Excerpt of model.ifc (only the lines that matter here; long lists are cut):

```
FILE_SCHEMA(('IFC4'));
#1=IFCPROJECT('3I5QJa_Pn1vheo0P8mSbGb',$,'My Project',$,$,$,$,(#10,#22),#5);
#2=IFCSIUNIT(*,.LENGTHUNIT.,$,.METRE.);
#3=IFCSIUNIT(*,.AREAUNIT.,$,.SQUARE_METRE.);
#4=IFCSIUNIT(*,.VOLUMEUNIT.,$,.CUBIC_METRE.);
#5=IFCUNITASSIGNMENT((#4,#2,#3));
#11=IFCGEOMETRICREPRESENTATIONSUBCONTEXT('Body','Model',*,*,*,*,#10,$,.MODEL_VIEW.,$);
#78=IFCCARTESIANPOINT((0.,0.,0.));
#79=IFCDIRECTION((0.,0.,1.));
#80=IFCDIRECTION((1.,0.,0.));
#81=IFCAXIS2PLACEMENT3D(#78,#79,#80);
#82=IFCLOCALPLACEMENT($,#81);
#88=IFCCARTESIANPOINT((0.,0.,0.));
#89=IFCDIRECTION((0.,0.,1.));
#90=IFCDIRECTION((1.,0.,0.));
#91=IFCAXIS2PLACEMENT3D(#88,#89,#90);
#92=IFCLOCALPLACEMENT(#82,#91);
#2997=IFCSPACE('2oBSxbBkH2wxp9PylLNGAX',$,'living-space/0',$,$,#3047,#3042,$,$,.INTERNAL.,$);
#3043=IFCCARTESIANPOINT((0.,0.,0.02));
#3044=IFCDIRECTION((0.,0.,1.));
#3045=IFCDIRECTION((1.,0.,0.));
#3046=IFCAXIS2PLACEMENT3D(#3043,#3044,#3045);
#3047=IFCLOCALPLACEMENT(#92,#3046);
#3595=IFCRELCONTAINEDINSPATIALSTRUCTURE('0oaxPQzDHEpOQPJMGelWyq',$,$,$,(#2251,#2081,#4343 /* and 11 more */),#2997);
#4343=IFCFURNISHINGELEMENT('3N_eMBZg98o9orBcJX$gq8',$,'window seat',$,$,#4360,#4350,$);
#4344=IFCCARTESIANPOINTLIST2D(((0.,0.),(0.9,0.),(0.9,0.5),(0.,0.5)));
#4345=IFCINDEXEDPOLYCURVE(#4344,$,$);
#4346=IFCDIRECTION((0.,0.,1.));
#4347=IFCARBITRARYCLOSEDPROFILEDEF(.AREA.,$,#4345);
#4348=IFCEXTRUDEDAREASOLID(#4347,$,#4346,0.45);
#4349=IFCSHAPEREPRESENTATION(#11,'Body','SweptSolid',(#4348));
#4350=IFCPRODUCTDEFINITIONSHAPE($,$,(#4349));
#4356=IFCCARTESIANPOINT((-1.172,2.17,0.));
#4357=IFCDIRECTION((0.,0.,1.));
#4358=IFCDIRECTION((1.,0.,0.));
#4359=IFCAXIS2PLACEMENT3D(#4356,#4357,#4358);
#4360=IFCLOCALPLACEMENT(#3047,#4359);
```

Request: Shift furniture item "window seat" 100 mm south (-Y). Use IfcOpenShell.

```python
import ifcopenshell
import ifcopenshell.api.geometry
import ifcopenshell.util.placement

model = ifcopenshell.open("model.ifc")

item = model.by_id(4343)
matrix = ifcopenshell.util.placement.get_local_placement(item.ObjectPlacement)
matrix[1, 3] -= 0.1
ifcopenshell.api.geometry.edit_object_placement(model, product=item, matrix=matrix, is_si=False)

print(ifcopenshell.util.placement.get_local_placement(item.ObjectPlacement).round(3) + 0.0)

model.write("model-out.ifc")
```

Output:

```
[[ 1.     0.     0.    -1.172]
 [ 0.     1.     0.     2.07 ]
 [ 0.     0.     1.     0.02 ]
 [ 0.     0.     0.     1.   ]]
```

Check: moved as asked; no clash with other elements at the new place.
